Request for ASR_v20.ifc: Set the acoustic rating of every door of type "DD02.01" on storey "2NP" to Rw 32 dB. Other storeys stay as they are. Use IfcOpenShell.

First a look at what the model holds.

```python
import ifcopenshell
import ifcopenshell.util.element

model = ifcopenshell.open("ASR_v20.ifc")
print(model.schema)
storey = next(s for s in model.by_type("IfcBuildingStorey") if s.Name == "2NP")
doors = [e for e in ifcopenshell.util.element.get_decomposition(storey) if e.is_a("IfcDoor")]
seen = {}
for e in doors:
    element_type = ifcopenshell.util.element.get_type(e)
    key = (element_type.Name if element_type != e and element_type else None, ifcopenshell.util.element.get_pset(e, "Pset_DoorCommon", "AcousticRating"))
    seen[key] = seen.get(key, 0) + 1
for (name, value), count in sorted(seen.items(), key=str):
    print(count, "x", name, "|", value)
```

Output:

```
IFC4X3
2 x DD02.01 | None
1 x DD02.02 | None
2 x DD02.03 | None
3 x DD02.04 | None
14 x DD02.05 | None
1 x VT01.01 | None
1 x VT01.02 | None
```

```python
import ifcopenshell
import ifcopenshell.api.pset
import ifcopenshell.util.element

model = ifcopenshell.open("ASR_v20.ifc")

storey = next(s for s in model.by_type("IfcBuildingStorey") if s.Name == "2NP")
doors = [e for e in ifcopenshell.util.element.get_decomposition(storey) if e.is_a("IfcDoor")]

count = 0
for e in doors:
    element_type = ifcopenshell.util.element.get_type(e)
    if element_type in (None, e) or element_type.Name != "DD02.01":
        continue
    # add_pset returns the element's existing set when there is one.
    pset = ifcopenshell.api.pset.add_pset(model, product=e, name="Pset_DoorCommon")
    ifcopenshell.api.pset.edit_pset(model, pset=pset, properties={"AcousticRating": "Rw 32 dB"})
    count += 1

print(count, "doors updated")

model.write("ASR_v20_v2.ifc")
```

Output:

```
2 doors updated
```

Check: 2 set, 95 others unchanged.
